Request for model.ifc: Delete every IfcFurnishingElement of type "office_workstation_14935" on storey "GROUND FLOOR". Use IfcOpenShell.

First a look at what the model holds.

```python
import ifcopenshell
import ifcopenshell.util.element

model = ifcopenshell.open("model.ifc")
print(model.schema)
storey = next(s for s in model.by_type("IfcBuildingStorey") if s.Name == "GROUND FLOOR")
furniture = [e for e in ifcopenshell.util.element.get_decomposition(storey) if e.is_a("IfcFurnishingElement")]
seen = {}
for e in furniture:
    element_type = ifcopenshell.util.element.get_type(e)
    name = element_type.Name if element_type not in (None, e) else None
    seen[name] = seen.get(name, 0) + 1
for name, count in sorted(seen.items(), key=str):
    print(count, "x", name)
```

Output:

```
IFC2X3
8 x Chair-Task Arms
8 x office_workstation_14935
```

```python
import ifcopenshell
import ifcopenshell.api.root
import ifcopenshell.util.element

model = ifcopenshell.open("model.ifc")

storey = next(s for s in model.by_type("IfcBuildingStorey") if s.Name == "GROUND FLOOR")
furniture = [e for e in ifcopenshell.util.element.get_decomposition(storey) if e.is_a("IfcFurnishingElement")]
targets = [e for e in furniture if (t := ifcopenshell.util.element.get_type(e)) not in (None, e) and t.Name == "office_workstation_14935"]

for e in targets:
    ifcopenshell.api.root.remove_product(model, product=e)
print(len(targets), "removed")

model.write("model_updated.ifc")
```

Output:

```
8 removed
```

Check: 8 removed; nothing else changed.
